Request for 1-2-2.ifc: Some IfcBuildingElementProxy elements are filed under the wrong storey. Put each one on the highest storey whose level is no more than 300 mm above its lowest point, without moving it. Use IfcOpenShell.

First a look at what the model holds.

```python
import ifcopenshell
import ifcopenshell.util.element
import ifcopenshell.util.placement

model = ifcopenshell.open("1-2-2.ifc")
print(model.schema)
for storey in model.by_type("IfcBuildingStorey"):
    level = ifcopenshell.util.placement.get_storey_elevation(storey)
    count = sum(e.is_a("IfcBuildingElementProxy") for e in ifcopenshell.util.element.get_contained(storey))
    print(storey.id(), storey.Name, round(level, 3), count, sep=" | ")
```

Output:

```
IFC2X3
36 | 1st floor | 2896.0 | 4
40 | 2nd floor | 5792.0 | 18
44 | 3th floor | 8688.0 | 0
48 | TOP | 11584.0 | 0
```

```python
import ifcopenshell
import ifcopenshell.api.spatial
import ifcopenshell.geom
import ifcopenshell.util.element
import ifcopenshell.util.placement
import ifcopenshell.util.shape
import ifcopenshell.util.unit

model = ifcopenshell.open("1-2-2.ifc")
unit_scale = ifcopenshell.util.unit.calculate_unit_scale(model)
settings = ifcopenshell.geom.settings()

levels = sorted(
    ((ifcopenshell.util.placement.get_storey_elevation(s) * unit_scale, s) for s in model.by_type("IfcBuildingStorey")),
    key=lambda pair: pair[0],
)

for e in model.by_type("IfcBuildingElementProxy"):
    current = e.ContainedInStructure[0].RelatingStructure if e.ContainedInStructure else None
    if current is None or not current.is_a("IfcBuildingStorey"):
        continue
    shape = ifcopenshell.geom.create_shape(settings, e)
    bottom = ifcopenshell.util.shape.get_shape_bottom_elevation(shape, shape.geometry)
    below = [s for level, s in levels if level <= bottom + 0.3]
    storey = below[-1] if below else levels[0][1]
    if storey != current:
        # assign_container keeps the world position.
        ifcopenshell.api.spatial.assign_container(model, products=[e], relating_structure=storey)
        print(e.id(), current.Name, "->", storey.Name)

model.write("1-2-2_rev.ifc")
```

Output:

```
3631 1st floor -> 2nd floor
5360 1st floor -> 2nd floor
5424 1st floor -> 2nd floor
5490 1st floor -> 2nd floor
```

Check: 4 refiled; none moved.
